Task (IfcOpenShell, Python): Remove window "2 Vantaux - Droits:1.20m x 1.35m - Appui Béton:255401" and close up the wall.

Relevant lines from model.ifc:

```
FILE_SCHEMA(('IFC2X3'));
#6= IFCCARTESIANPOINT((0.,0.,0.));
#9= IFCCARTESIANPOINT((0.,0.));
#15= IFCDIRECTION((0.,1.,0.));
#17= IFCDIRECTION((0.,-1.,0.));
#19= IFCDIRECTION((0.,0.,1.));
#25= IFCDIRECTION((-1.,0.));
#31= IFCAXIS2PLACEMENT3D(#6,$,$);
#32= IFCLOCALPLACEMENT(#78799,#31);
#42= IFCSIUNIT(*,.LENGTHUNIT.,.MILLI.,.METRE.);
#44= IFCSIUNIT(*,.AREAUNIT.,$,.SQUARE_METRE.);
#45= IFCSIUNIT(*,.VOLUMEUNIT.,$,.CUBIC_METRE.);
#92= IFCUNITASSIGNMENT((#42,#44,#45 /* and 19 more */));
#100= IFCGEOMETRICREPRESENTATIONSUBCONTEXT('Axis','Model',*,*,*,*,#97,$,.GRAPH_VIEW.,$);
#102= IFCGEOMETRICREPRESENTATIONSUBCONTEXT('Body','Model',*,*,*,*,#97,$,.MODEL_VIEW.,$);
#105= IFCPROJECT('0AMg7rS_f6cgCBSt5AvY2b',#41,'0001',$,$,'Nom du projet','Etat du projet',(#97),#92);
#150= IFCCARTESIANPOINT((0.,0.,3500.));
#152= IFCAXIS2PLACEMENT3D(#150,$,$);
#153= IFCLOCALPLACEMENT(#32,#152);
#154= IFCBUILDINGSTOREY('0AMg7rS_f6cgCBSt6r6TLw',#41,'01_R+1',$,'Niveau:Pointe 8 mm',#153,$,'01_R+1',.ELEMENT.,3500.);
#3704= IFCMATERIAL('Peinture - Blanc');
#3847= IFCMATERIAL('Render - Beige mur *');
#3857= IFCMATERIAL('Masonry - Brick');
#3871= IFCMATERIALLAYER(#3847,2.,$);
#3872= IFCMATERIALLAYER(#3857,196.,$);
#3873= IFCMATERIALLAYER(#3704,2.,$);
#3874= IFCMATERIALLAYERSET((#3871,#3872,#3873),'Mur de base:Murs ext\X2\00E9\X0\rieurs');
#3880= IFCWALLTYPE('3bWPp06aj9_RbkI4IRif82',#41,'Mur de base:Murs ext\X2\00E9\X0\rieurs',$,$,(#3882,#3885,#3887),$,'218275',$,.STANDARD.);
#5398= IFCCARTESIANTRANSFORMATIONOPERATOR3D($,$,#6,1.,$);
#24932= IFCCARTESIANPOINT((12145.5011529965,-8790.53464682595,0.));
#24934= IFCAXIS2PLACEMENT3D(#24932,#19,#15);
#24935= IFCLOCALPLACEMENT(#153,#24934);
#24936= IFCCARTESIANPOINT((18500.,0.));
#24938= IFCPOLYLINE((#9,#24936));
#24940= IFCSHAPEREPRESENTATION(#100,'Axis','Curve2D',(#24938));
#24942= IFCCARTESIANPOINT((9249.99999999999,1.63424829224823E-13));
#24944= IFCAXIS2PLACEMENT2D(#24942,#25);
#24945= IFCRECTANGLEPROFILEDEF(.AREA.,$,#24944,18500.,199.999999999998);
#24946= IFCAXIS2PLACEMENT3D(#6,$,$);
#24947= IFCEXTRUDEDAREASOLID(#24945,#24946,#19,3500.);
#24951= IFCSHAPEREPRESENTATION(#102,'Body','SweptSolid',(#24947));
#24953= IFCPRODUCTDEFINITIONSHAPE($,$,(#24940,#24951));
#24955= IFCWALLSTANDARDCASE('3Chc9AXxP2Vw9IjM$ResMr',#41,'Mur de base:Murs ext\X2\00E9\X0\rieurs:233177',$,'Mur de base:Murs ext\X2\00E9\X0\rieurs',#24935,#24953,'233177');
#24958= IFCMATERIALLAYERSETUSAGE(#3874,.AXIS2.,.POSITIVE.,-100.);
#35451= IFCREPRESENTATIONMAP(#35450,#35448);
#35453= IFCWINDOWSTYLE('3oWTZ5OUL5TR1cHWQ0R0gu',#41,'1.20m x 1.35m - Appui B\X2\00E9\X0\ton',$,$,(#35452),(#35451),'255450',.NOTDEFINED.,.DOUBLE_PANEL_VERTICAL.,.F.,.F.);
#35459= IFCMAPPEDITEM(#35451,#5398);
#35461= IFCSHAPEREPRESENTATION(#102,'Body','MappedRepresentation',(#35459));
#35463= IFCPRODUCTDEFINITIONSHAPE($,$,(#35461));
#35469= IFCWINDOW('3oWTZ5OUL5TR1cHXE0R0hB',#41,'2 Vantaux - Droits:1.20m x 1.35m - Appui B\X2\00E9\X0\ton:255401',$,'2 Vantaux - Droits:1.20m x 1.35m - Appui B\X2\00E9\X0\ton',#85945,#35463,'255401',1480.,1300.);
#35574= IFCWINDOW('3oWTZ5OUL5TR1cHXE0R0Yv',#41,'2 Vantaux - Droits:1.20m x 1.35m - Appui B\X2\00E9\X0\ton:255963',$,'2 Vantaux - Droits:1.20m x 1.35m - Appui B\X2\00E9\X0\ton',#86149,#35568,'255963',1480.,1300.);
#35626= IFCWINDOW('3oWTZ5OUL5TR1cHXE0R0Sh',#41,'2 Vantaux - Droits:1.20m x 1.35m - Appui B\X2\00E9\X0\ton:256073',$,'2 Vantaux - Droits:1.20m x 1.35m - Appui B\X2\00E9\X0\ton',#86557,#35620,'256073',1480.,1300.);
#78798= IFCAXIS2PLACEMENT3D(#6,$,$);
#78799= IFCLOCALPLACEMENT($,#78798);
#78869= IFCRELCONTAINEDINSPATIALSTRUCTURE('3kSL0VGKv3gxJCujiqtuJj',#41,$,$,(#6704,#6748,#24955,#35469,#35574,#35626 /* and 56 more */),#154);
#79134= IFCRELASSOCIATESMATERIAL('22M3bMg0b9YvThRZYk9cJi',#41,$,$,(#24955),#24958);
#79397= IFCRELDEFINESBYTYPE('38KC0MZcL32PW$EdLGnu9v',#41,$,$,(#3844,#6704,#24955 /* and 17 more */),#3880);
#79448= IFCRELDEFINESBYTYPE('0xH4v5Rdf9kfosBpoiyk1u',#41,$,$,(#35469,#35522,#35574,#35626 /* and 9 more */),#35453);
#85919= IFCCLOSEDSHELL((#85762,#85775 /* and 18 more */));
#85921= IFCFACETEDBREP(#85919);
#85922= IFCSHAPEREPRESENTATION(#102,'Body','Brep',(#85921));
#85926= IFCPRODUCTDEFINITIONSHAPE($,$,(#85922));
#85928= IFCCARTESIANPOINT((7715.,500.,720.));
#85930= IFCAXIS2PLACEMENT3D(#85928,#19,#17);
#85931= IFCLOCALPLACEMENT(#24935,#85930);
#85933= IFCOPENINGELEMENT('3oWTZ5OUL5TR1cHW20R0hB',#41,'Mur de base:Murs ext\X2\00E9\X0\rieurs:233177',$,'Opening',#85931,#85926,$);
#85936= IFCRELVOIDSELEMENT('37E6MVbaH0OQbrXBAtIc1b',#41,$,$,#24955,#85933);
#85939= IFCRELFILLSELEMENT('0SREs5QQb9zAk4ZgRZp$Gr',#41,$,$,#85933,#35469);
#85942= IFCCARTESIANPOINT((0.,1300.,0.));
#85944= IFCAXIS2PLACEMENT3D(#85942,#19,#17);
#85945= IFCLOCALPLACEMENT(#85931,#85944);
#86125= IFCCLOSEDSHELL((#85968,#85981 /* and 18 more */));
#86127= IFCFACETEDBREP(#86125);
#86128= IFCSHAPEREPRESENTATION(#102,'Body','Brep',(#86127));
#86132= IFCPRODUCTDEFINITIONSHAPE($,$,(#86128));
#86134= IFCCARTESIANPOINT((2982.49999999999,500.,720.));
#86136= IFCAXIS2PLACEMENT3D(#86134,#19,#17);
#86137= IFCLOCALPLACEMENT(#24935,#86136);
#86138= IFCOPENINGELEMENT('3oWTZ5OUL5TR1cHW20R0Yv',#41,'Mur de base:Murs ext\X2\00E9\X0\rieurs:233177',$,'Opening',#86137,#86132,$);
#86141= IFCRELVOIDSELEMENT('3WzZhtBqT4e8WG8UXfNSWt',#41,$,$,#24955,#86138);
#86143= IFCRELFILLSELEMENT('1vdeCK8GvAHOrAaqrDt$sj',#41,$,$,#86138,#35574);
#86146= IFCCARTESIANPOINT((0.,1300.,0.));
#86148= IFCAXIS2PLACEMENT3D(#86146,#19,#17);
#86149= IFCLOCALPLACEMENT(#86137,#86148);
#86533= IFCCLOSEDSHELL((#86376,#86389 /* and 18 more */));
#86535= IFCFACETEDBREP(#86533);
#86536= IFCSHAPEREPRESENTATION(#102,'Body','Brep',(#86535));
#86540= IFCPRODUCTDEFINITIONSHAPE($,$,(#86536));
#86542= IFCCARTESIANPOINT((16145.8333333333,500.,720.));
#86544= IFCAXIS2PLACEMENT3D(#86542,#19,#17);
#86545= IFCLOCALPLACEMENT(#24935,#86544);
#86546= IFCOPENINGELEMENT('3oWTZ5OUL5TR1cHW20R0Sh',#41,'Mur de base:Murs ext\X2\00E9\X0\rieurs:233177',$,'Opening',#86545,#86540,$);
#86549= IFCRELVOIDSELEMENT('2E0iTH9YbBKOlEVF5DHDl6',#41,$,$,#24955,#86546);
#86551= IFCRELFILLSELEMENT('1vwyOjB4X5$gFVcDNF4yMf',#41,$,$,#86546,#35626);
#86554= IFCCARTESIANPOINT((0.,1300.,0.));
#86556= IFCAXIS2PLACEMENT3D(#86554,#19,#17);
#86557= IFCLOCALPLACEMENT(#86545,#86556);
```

```python
import ifcopenshell
import ifcopenshell.api.feature
import ifcopenshell.api.root
import ifcopenshell.geom
import ifcopenshell.util.shape

model = ifcopenshell.open("model.ifc")
settings = ifcopenshell.geom.settings()


def volume(element):
    """Net volume in cubic metres, openings subtracted."""
    shape = ifcopenshell.geom.create_shape(settings, element)
    return ifcopenshell.util.shape.get_volume(shape.geometry)


window = model.by_id(35469)
opening = window.FillsVoids[0].RelatingOpeningElement
wall = opening.VoidsElements[0].RelatingBuildingElement
before = volume(wall)

ifcopenshell.api.root.remove_product(model, product=window)
ifcopenshell.api.feature.remove_feature(model, feature=opening)

after = volume(wall)

print(f"wall volume {before:.3f} -> {after:.3f} m3")

model.write("model_v2.ifc")
```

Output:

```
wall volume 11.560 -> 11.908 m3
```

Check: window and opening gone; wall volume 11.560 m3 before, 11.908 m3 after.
